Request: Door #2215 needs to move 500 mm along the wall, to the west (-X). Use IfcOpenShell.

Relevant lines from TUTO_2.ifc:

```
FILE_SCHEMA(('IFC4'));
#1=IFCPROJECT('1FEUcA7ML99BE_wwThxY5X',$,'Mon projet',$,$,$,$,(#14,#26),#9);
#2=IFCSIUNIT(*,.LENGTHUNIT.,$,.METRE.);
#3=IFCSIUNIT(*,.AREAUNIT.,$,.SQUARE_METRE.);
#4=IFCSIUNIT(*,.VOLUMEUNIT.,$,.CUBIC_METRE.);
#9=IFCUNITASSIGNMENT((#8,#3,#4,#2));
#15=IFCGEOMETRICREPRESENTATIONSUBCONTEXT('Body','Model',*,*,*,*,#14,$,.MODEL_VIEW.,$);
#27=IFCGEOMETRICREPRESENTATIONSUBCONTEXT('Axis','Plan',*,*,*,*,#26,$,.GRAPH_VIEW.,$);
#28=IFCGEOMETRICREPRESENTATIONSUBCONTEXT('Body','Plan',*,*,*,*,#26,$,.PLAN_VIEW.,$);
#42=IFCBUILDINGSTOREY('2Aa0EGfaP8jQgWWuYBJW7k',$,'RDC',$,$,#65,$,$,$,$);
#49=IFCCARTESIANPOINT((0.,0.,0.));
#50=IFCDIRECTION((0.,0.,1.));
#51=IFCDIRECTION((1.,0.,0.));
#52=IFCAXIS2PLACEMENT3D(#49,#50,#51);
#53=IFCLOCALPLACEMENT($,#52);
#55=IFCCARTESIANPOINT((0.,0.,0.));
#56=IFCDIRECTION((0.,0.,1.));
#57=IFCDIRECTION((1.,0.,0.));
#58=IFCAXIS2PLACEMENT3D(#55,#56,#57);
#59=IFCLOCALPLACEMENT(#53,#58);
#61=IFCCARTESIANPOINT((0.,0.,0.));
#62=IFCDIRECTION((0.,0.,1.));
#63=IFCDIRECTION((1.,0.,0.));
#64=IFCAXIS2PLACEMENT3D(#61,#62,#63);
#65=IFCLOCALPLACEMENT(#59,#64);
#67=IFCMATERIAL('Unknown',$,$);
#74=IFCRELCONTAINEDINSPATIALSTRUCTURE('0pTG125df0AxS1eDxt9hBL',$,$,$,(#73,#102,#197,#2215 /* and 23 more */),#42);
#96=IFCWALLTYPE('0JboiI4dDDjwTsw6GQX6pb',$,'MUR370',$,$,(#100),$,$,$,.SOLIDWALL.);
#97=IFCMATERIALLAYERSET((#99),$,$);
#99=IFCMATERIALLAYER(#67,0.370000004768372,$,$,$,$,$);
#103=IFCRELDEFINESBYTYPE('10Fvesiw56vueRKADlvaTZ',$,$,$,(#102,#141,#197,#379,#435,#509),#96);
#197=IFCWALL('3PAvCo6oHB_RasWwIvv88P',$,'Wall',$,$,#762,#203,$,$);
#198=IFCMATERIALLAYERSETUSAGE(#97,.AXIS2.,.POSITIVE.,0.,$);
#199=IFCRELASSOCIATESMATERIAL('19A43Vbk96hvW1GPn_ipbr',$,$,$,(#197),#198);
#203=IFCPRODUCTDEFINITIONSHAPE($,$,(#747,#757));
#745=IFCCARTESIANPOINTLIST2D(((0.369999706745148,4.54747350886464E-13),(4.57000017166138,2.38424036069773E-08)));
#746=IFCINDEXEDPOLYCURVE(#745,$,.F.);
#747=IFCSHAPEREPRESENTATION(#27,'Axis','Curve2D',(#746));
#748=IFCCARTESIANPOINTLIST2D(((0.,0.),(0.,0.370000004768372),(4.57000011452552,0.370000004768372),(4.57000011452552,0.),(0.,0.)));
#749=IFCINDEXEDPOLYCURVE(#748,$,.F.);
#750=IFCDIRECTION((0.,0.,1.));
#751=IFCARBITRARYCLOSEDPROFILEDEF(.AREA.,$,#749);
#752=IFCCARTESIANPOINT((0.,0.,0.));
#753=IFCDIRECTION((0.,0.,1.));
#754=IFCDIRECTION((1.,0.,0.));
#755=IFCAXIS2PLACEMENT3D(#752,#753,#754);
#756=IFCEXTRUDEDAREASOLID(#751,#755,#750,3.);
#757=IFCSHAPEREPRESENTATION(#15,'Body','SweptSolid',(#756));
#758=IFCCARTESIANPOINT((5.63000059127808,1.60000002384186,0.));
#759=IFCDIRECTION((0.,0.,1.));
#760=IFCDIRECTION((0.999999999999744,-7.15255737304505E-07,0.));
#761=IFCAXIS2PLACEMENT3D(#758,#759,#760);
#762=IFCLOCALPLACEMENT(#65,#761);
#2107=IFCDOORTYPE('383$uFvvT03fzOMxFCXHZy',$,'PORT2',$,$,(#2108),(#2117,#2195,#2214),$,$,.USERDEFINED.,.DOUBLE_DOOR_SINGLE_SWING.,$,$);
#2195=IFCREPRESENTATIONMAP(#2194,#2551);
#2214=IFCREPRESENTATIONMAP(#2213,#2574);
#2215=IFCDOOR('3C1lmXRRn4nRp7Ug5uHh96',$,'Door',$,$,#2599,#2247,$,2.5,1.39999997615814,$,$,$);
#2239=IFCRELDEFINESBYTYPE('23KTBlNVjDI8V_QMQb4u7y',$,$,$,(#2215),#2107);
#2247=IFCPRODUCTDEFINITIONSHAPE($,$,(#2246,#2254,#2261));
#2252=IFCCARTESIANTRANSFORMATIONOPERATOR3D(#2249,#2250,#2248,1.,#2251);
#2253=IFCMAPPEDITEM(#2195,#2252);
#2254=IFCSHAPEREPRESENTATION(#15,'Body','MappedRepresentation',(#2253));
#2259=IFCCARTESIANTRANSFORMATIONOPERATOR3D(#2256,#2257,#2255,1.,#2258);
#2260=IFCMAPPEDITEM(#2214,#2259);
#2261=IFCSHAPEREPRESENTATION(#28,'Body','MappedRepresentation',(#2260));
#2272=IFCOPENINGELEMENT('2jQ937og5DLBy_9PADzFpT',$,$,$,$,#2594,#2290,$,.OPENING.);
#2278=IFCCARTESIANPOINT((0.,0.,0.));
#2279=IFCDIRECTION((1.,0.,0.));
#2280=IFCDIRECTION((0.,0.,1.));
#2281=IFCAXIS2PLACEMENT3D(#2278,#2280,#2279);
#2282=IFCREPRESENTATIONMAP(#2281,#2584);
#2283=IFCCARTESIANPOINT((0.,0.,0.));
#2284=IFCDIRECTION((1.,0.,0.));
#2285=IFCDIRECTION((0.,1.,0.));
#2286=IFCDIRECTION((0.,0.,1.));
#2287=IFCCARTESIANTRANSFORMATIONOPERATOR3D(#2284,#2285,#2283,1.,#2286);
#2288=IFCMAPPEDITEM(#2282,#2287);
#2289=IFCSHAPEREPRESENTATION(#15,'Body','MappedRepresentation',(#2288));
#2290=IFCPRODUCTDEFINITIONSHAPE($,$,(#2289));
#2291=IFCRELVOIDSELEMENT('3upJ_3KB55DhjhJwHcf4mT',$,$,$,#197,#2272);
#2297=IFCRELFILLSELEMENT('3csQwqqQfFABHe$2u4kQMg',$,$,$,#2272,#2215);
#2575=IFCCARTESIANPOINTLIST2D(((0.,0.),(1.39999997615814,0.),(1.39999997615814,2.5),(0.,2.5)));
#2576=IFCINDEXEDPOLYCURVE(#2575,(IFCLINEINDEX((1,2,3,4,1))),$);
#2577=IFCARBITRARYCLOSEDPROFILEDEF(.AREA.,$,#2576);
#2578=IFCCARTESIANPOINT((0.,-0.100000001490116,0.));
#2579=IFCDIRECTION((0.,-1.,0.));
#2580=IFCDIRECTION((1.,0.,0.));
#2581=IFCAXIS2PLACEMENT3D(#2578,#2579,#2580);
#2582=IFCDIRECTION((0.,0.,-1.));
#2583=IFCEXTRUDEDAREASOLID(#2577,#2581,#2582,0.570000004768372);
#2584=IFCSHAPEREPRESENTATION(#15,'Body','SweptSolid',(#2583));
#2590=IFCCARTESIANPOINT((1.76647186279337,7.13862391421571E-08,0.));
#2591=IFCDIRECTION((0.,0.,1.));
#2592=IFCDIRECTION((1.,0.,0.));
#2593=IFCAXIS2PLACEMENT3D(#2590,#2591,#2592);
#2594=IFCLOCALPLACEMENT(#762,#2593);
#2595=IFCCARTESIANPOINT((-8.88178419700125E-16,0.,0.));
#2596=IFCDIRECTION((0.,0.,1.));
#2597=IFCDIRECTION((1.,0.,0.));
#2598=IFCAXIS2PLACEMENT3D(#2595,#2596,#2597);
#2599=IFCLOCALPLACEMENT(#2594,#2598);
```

```python
import ifcopenshell
import ifcopenshell.api.geometry
import ifcopenshell.util.placement
import ifcopenshell.util.unit

model = ifcopenshell.open("TUTO_2.ifc")
unit_scale = ifcopenshell.util.unit.calculate_unit_scale(model)

door = model.by_guid("3C1lmXRRn4nRp7Ug5uHh96")
opening = door.FillsVoids[0].RelatingOpeningElement
wall = opening.VoidsElements[0].RelatingBuildingElement

wall_matrix = ifcopenshell.util.placement.get_local_placement(wall.ObjectPlacement)
shift = wall_matrix[:3, 0] * -0.5 / unit_scale
before = ifcopenshell.util.placement.get_local_placement(door.ObjectPlacement)[:3, 3].copy()

# The door is placed relative to its opening, so it follows when the opening moves.
matrix = ifcopenshell.util.placement.get_local_placement(opening.ObjectPlacement)
matrix[:3, 3] += shift
ifcopenshell.api.geometry.edit_object_placement(
    model, product=opening, matrix=matrix, is_si=False, should_transform_children=True
)

after = ifcopenshell.util.placement.get_local_placement(door.ObjectPlacement)[:3, 3]
print("door moved by", (after - before).round(3) + 0.0)

model.write("TUTO_2-out.ifc")
```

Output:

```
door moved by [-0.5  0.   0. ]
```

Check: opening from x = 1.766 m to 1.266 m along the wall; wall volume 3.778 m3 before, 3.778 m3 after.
